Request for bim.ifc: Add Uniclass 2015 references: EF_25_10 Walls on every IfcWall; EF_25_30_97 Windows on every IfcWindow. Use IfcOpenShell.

First a look at what the model holds.

```python
import ifcopenshell

model = ifcopenshell.open("bim.ifc")
print(model.schema)
print("classifications:", [c.Name for c in model.by_type("IfcClassification")])
for ifc_class in ("IfcDoor", "IfcRoof", "IfcStair", "IfcWall", "IfcWindow"):
    print(ifc_class, len(model.by_type(ifc_class)))
```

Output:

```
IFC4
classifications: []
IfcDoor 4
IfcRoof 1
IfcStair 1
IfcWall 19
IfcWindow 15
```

```python
import ifcopenshell
import ifcopenshell.api.classification

model = ifcopenshell.open("bim.ifc")

system = ifcopenshell.api.classification.add_classification(model, classification="Uniclass 2015")

codes = {
    "IfcWall": ("EF_25_10", "Walls"),
    "IfcWindow": ("EF_25_30_97", "Windows"),
}
for ifc_class, (code, name) in codes.items():
    products = model.by_type(ifc_class)
    ifcopenshell.api.classification.add_reference(
        model, products=products, classification=system, identification=code, name=name
    )
    print(code, len(products))

model.write("bim_v2.ifc")
```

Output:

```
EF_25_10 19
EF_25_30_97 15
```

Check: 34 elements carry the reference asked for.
